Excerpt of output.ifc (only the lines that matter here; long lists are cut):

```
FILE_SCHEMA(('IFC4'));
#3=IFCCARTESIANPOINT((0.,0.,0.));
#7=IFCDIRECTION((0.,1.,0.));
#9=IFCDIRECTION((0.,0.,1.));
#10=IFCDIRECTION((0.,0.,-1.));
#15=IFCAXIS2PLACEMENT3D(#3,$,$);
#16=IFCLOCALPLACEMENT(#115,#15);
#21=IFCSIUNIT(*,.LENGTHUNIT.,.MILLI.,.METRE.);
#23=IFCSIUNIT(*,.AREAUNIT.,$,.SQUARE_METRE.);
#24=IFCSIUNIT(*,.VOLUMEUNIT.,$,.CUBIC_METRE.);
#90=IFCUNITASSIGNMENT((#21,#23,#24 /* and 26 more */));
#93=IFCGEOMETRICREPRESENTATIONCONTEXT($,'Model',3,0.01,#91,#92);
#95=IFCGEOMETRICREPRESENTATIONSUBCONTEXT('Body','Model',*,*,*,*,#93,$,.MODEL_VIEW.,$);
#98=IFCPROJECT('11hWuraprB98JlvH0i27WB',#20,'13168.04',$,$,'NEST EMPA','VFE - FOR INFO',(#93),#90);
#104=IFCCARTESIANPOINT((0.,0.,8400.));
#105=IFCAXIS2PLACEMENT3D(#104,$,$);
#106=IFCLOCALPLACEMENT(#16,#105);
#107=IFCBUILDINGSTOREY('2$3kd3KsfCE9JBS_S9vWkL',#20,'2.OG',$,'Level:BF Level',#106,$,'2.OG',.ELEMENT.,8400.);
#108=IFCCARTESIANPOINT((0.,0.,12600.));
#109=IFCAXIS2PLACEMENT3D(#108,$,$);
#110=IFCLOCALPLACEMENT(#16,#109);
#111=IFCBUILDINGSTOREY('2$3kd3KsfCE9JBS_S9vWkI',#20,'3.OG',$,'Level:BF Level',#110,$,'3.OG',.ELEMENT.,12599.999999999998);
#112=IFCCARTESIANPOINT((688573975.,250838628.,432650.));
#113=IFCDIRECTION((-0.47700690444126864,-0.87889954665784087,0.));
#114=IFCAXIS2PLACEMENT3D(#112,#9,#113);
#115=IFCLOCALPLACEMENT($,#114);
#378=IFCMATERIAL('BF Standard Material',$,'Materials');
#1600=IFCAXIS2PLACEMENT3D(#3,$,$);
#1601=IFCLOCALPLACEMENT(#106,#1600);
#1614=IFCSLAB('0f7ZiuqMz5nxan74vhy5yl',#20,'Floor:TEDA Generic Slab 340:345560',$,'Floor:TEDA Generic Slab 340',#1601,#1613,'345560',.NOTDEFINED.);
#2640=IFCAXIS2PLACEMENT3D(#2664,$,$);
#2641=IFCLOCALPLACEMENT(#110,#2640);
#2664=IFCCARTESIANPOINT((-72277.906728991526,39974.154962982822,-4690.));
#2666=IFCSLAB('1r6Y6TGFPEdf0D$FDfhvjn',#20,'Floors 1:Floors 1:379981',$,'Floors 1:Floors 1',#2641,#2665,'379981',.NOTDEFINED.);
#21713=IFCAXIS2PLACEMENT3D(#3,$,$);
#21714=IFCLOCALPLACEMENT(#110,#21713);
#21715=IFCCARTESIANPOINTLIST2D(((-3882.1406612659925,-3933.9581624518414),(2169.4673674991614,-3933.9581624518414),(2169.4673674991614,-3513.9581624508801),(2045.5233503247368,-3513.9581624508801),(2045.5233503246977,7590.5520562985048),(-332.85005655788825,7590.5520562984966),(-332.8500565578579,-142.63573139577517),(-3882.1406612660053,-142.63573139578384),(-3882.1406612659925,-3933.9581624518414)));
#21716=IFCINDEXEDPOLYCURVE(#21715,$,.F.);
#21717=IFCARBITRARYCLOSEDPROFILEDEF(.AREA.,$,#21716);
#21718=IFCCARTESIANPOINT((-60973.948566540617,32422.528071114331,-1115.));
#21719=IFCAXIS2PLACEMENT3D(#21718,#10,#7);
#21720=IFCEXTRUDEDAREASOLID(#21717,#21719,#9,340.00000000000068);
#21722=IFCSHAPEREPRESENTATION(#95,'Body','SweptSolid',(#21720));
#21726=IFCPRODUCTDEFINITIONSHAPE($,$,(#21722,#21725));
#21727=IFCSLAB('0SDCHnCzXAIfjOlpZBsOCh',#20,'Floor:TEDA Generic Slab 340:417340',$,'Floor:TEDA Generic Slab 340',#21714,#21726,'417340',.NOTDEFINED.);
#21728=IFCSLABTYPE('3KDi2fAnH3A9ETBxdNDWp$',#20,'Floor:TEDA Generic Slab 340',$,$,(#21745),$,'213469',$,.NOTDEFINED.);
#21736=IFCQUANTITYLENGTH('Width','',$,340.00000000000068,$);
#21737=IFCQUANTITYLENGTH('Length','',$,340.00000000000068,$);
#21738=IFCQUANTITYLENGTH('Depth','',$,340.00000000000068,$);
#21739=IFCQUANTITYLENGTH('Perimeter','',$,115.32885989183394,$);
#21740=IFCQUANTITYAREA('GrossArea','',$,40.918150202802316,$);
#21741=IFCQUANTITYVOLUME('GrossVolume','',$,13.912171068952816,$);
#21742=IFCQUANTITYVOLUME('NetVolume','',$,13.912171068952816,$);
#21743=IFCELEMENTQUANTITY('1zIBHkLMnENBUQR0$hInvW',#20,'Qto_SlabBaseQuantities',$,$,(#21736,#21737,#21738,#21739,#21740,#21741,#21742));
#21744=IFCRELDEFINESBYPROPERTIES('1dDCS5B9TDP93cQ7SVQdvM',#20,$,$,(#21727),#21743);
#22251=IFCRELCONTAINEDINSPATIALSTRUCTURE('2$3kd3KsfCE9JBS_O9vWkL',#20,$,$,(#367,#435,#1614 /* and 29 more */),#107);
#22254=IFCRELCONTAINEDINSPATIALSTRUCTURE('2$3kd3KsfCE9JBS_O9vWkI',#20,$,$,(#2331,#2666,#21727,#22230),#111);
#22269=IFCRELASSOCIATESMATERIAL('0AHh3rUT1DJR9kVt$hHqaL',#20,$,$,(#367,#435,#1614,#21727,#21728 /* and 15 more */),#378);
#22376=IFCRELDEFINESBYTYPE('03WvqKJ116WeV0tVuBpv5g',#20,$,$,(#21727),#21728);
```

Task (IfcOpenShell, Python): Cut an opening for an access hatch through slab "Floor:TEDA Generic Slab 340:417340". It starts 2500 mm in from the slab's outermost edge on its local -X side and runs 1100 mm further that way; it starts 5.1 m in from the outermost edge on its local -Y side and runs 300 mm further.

```python
import numpy as np
import ifcopenshell
import ifcopenshell.api.feature
import ifcopenshell.api.geometry
import ifcopenshell.api.pset
import ifcopenshell.api.root
import ifcopenshell.geom
import ifcopenshell.util.element
import ifcopenshell.util.placement
import ifcopenshell.util.representation
import ifcopenshell.util.shape
import ifcopenshell.util.unit

model = ifcopenshell.open("output.ifc")
unit_scale = ifcopenshell.util.unit.calculate_unit_scale(model)
volume_scale = ifcopenshell.util.unit.calculate_unit_scale(model, "VOLUMEUNIT")
settings = ifcopenshell.geom.settings()


def volume(element):
    """Net volume in cubic metres, openings subtracted."""
    shape = ifcopenshell.geom.create_shape(settings, element)
    return ifcopenshell.util.shape.get_volume(shape.geometry)


slab = model.by_id(21727)
before = volume(slab)

# Extent in the slab's own axes, in metres. The edges named are its -X and -Y sides.
slab_shape = ifcopenshell.geom.create_shape(settings, slab)
vertices = ifcopenshell.util.shape.get_vertices(slab_shape.geometry)
x_min, y_min, bottom = vertices.min(axis=0)
top = vertices[:, 2].max()

opening = ifcopenshell.api.root.create_entity(model, ifc_class="IfcOpeningElement", name="Access hatch opening", predefined_type="OPENING")
context = ifcopenshell.util.representation.get_context(model, "Model", "Body", "MODEL_VIEW")
width, depth = 1.1, 0.3
outline = [(0.0, 0.0), (width, 0.0), (width, depth), (0.0, depth), (0.0, 0.0)]
# Overshoot both faces by 50 mm so the cut is clean.
shape = ifcopenshell.api.geometry.add_slab_representation(
    model, context=context, depth=top - bottom + 0.1, polyline=outline
)
ifcopenshell.api.geometry.assign_representation(model, product=opening, representation=shape)

matrix = ifcopenshell.util.placement.get_local_placement(slab.ObjectPlacement)
matrix[:, 3] = matrix @ np.append(np.array([x_min + 2.5, y_min + 5.1, bottom - 0.05]) / unit_scale, 1.0)
ifcopenshell.api.geometry.edit_object_placement(model, product=opening, matrix=matrix, is_si=False)
ifcopenshell.api.feature.add_feature(model, feature=opening, element=slab)

after = volume(slab)

# Update the slab's stored quantities.
qto = model.by_id(ifcopenshell.util.element.get_pset(slab, "Qto_SlabBaseQuantities", should_inherit=False)["id"])
ifcopenshell.api.pset.edit_qto(model, qto=qto, properties={"NetVolume": after / volume_scale})

print(f"slab volume {before:.3f} -> {after:.3f} m3")

model.write("output_updated.ifc")
```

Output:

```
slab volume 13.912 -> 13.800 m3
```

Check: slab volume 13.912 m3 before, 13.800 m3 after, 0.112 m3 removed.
